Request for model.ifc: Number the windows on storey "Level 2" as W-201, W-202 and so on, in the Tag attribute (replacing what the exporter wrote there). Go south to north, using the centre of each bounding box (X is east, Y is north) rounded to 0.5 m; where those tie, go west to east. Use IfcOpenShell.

First a look at what the model holds.

```python
import ifcopenshell
import ifcopenshell.util.element
import ifcopenshell.util.placement

model = ifcopenshell.open("model.ifc")
print(model.schema)
storey = next(s for s in model.by_type("IfcBuildingStorey") if s.Name == "Level 2")
windows = [e for e in ifcopenshell.util.element.get_decomposition(storey) if e.is_a("IfcWindow")]
for e in sorted(windows, key=lambda e: e.id()):
    origin = ifcopenshell.util.placement.get_local_placement(e.ObjectPlacement)[:3, 3]
    print(e.id(), e.Tag, e.Name, origin.round(2) + 0.0, sep=" | ")
```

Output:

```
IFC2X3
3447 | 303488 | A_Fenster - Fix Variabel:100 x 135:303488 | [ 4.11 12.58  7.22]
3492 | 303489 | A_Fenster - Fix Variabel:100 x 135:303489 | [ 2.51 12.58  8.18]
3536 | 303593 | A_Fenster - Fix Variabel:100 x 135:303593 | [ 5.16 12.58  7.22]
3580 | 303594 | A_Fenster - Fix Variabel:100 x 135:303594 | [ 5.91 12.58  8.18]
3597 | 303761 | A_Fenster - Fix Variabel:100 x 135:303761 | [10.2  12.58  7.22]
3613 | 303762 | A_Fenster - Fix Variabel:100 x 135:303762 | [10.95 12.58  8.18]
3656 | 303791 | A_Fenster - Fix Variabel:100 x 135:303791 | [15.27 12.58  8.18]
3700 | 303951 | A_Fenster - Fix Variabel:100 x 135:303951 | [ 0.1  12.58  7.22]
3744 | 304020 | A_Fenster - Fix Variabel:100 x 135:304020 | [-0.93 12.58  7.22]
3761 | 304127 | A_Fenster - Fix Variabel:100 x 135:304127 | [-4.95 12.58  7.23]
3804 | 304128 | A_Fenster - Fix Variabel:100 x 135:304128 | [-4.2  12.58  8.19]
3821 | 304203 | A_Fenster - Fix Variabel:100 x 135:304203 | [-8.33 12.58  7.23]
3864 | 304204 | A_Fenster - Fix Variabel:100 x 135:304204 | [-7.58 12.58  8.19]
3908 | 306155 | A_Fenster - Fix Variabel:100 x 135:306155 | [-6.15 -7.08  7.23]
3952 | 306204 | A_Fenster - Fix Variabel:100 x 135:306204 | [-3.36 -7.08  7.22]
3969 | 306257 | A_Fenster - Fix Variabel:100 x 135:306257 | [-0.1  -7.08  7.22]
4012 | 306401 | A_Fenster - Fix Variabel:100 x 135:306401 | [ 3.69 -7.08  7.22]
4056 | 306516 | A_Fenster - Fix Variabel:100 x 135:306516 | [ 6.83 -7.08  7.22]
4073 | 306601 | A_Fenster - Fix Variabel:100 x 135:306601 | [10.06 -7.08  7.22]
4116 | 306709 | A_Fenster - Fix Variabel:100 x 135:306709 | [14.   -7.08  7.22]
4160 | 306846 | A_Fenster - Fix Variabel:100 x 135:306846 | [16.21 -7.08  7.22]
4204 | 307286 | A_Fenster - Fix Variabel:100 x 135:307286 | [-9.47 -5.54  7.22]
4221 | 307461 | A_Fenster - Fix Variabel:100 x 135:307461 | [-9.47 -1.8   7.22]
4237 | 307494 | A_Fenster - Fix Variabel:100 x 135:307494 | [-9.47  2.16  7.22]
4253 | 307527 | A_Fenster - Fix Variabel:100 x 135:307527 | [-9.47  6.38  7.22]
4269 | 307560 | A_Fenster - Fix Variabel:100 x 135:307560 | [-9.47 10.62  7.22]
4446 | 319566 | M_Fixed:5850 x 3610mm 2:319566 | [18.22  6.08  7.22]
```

```python
import ifcopenshell
import ifcopenshell.geom
import ifcopenshell.util.element
import ifcopenshell.util.shape

model = ifcopenshell.open("model.ifc")
settings = ifcopenshell.geom.settings()
settings.set("use-world-coords", True)


def centre(element):
    shape = ifcopenshell.geom.create_shape(settings, element)
    return ifcopenshell.util.shape.get_bbox_centroid(shape.geometry)


storey = next(s for s in model.by_type("IfcBuildingStorey") if s.Name == "Level 2")
windows = [e for e in ifcopenshell.util.element.get_decomposition(storey) if e.is_a("IfcWindow")]

# Insertion points can sit at a corner or the storey origin, so sort by the geometry (in metres).
centres = {e: centre(e) for e in windows}
windows.sort(key=lambda e: (round(centres[e][1] / 0.5), centres[e][0]))

for i, e in enumerate(windows, start=1):
    number = f"W-2{i:02d}"
    e.Tag = number
    print(e.id(), number)

model.write("model-out.ifc")
```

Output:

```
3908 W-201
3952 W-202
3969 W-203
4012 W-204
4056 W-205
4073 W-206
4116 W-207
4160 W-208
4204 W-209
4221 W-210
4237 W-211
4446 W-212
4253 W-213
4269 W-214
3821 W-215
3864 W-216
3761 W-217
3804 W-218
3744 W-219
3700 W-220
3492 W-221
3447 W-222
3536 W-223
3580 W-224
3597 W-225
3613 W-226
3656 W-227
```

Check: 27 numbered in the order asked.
